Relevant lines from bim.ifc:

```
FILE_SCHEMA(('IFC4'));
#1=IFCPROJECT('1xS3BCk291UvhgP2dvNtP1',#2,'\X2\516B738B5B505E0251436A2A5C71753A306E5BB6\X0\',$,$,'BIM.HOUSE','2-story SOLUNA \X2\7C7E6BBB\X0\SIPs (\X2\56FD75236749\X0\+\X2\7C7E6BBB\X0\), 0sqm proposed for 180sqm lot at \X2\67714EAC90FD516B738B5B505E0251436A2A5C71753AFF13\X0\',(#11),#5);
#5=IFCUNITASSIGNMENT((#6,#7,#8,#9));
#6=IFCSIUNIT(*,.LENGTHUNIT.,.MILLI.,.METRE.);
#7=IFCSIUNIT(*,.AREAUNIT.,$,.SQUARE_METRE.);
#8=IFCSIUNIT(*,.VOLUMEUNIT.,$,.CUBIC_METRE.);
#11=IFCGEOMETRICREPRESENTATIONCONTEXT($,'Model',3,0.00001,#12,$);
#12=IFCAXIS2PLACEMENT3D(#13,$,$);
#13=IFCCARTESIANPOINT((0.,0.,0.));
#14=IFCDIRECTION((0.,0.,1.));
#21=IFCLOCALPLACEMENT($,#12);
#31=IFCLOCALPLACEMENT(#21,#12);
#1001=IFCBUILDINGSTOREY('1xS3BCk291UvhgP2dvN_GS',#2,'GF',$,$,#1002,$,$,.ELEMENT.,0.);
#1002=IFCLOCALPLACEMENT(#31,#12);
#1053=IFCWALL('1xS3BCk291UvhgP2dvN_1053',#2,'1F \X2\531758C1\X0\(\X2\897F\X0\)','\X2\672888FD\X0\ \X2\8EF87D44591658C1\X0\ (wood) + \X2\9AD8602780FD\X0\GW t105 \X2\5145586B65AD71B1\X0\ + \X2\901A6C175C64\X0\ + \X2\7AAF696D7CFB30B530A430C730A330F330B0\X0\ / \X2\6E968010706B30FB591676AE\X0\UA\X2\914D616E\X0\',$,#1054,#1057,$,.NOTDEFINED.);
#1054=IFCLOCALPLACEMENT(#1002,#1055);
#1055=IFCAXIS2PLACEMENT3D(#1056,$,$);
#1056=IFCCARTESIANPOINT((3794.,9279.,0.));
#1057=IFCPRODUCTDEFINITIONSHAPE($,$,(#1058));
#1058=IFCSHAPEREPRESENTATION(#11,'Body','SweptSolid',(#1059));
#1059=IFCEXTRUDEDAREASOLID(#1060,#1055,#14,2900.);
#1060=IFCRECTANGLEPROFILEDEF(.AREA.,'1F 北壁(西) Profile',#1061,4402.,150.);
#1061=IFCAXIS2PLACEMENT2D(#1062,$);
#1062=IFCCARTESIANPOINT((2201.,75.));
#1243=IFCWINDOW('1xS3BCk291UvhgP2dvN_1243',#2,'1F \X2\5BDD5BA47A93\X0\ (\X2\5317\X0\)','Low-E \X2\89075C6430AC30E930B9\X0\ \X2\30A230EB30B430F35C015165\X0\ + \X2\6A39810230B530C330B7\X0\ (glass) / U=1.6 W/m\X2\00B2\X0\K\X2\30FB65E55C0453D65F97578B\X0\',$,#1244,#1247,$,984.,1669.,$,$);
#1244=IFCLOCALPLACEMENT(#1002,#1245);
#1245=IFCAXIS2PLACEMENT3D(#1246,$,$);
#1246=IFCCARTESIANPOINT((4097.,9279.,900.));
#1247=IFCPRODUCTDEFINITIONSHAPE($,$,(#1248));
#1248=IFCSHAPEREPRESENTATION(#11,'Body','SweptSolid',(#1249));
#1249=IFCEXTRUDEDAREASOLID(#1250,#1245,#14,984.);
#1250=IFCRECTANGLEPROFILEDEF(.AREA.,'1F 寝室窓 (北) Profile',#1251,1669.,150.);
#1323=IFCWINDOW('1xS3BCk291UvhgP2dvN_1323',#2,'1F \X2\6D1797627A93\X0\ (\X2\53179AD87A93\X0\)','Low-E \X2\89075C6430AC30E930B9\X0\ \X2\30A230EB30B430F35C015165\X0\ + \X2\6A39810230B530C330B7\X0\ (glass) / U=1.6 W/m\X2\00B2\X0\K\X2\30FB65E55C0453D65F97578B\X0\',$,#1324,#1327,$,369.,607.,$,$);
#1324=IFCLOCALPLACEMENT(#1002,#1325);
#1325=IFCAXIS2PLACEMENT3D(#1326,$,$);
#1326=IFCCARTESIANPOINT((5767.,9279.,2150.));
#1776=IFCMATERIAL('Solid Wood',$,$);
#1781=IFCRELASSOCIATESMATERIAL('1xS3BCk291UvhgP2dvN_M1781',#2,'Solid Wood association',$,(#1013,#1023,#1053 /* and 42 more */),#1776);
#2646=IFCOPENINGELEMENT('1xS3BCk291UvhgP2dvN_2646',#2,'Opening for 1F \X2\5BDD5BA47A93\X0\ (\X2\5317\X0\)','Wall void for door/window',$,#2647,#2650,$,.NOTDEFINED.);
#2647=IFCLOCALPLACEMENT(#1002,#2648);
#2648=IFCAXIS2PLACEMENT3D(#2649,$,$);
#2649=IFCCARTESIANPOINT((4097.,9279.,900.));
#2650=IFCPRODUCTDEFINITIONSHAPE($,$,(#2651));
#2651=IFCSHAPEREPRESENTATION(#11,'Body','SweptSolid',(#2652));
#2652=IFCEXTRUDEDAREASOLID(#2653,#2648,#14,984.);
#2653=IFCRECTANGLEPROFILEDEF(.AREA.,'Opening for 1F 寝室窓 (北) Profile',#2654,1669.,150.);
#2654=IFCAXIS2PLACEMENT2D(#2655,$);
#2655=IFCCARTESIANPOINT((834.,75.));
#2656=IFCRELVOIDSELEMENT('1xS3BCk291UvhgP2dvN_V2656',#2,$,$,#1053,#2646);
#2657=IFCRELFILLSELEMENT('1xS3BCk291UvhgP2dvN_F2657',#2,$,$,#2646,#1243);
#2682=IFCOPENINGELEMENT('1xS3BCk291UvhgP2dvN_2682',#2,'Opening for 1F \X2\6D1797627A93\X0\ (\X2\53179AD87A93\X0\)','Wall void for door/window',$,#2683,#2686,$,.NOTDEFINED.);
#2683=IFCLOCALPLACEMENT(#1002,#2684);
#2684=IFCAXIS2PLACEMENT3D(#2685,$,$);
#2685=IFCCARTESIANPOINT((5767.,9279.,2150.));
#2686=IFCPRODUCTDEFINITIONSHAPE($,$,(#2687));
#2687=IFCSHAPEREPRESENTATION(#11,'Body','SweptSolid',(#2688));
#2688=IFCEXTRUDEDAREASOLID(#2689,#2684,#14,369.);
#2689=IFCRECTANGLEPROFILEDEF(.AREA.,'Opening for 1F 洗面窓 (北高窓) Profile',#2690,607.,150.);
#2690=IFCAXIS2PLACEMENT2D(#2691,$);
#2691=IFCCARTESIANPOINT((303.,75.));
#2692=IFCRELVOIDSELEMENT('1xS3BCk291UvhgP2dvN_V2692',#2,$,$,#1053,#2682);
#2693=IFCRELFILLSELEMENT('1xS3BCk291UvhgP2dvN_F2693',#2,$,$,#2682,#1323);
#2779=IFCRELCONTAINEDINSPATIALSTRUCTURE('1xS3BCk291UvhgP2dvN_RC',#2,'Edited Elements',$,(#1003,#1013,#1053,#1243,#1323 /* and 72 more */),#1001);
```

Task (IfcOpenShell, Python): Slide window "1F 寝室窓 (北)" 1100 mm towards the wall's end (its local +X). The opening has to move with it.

```python
import ifcopenshell
import ifcopenshell.api.geometry
import ifcopenshell.util.placement
import ifcopenshell.util.unit

model = ifcopenshell.open("bim.ifc")
unit_scale = ifcopenshell.util.unit.calculate_unit_scale(model)

window = model.by_guid("1xS3BCk291UvhgP2dvN_1243")
opening = window.FillsVoids[0].RelatingOpeningElement
wall = opening.VoidsElements[0].RelatingBuildingElement

wall_matrix = ifcopenshell.util.placement.get_local_placement(wall.ObjectPlacement)
shift = wall_matrix[:3, 0] * 1.1 / unit_scale
before = ifcopenshell.util.placement.get_local_placement(window.ObjectPlacement)[:3, 3].copy()

# The window is not placed relative to its opening, so move both.
for product in (opening, window):
    matrix = ifcopenshell.util.placement.get_local_placement(product.ObjectPlacement)
    matrix[:3, 3] += shift
    ifcopenshell.api.geometry.edit_object_placement(model, product=product, matrix=matrix, is_si=False)

after = ifcopenshell.util.placement.get_local_placement(window.ObjectPlacement)[:3, 3]
print("window moved by", (after - before).round(3) + 0.0)

model.write("bim_v2.ifc")
```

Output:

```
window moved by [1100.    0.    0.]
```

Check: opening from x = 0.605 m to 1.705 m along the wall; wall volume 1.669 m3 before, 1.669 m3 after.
